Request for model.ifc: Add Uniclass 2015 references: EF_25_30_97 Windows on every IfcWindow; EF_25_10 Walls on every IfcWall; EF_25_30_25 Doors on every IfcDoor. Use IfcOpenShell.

First a look at what the model holds.

```python
import ifcopenshell

model = ifcopenshell.open("model.ifc")
print(model.schema)
print("classifications:", [c.Name for c in model.by_type("IfcClassification")])
for ifc_class in ("IfcDoor", "IfcRoof", "IfcStair", "IfcWall", "IfcWindow"):
    print(ifc_class, len(model.by_type(ifc_class)))
```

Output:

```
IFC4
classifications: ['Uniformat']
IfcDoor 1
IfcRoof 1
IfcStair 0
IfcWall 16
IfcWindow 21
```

```python
import ifcopenshell
import ifcopenshell.api.classification

model = ifcopenshell.open("model.ifc")

system = ifcopenshell.api.classification.add_classification(model, classification="Uniclass 2015")

codes = {
    "IfcWindow": ("EF_25_30_97", "Windows"),
    "IfcWall": ("EF_25_10", "Walls"),
    "IfcDoor": ("EF_25_30_25", "Doors"),
}
for ifc_class, (code, name) in codes.items():
    products = model.by_type(ifc_class)
    ifcopenshell.api.classification.add_reference(
        model, products=products, classification=system, identification=code, name=name
    )
    print(code, len(products))

model.write("model_updated.ifc")
```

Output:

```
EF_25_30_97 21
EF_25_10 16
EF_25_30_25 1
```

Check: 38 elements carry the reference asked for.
